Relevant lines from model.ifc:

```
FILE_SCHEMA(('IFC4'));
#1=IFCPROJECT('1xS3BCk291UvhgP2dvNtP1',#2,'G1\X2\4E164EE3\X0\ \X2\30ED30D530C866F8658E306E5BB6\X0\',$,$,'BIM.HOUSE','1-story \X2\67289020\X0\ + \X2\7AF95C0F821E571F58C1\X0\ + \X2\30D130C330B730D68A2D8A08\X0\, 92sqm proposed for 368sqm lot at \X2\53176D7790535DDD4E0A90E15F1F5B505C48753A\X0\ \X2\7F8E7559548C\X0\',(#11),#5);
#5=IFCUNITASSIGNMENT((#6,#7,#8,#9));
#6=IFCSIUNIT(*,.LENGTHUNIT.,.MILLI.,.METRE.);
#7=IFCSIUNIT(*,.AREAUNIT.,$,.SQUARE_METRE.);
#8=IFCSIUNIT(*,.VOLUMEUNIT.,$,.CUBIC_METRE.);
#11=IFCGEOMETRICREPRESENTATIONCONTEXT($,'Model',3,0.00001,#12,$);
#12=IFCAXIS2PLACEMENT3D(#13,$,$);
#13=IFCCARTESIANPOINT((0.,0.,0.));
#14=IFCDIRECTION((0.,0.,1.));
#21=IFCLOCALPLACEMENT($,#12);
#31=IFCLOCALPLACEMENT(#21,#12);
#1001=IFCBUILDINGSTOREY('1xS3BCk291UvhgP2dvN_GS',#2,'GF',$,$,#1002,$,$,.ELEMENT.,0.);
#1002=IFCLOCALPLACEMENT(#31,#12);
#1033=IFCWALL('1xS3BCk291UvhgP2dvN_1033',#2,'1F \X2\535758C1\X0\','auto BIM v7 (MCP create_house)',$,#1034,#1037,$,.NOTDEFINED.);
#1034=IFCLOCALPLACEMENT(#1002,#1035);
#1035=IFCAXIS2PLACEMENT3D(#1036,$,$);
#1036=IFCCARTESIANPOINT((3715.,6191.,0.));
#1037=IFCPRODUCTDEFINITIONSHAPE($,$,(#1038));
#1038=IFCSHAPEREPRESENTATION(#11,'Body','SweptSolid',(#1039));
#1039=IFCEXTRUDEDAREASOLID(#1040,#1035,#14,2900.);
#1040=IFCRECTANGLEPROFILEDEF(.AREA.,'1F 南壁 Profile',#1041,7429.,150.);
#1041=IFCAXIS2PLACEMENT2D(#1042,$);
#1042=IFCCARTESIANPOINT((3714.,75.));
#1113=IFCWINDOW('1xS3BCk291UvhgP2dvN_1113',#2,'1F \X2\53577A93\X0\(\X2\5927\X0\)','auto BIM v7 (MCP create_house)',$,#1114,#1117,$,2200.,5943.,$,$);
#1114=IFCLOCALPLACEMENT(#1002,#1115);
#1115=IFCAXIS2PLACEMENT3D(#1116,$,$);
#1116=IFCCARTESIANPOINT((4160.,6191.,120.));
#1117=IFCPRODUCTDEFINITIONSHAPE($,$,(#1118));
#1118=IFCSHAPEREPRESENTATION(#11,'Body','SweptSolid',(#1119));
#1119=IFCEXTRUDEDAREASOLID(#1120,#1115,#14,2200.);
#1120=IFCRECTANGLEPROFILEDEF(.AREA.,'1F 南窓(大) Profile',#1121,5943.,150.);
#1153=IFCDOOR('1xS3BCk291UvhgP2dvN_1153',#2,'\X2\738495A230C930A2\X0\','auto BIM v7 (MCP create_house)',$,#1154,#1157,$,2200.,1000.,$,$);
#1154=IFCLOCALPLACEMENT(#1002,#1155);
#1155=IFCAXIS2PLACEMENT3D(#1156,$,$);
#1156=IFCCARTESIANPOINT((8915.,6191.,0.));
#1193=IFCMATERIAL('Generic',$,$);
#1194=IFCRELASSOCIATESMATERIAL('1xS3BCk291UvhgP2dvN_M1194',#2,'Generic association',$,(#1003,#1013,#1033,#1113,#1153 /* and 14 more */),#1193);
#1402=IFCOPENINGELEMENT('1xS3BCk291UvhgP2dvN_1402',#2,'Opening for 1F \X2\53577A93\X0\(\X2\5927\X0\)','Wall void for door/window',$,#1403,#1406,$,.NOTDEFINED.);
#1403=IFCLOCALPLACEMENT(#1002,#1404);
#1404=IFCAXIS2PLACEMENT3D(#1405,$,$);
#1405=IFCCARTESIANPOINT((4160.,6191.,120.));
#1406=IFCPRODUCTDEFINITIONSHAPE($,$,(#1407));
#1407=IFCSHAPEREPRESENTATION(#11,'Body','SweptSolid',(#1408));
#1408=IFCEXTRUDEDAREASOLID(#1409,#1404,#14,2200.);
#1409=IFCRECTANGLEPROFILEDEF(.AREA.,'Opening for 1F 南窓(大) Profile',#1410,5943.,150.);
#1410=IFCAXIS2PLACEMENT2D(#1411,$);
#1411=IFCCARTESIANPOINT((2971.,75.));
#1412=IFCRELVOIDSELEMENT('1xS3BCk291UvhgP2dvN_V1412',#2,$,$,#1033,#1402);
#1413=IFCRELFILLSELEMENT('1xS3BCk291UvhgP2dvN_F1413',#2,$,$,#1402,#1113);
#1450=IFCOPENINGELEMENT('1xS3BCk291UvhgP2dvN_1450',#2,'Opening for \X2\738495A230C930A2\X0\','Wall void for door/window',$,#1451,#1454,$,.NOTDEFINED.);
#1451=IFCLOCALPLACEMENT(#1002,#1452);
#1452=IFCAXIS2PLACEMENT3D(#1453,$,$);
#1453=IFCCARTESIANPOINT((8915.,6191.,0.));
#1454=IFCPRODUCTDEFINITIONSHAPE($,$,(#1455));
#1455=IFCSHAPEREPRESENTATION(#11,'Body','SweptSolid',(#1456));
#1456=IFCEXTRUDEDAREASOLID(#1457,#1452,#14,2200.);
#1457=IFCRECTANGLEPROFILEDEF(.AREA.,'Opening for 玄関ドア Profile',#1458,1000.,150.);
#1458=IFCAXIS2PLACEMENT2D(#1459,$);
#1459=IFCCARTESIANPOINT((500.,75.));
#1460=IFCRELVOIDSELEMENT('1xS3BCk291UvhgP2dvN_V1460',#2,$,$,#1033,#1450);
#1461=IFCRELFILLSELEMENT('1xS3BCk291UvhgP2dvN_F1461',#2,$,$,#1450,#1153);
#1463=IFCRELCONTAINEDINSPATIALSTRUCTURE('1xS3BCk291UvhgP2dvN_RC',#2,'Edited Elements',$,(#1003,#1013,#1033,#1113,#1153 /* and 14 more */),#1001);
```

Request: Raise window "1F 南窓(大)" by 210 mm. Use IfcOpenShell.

```python
import numpy as np
import ifcopenshell
import ifcopenshell.api.geometry
import ifcopenshell.util.placement
import ifcopenshell.util.unit

model = ifcopenshell.open("model.ifc")
unit_scale = ifcopenshell.util.unit.calculate_unit_scale(model)

window = model.by_guid("1xS3BCk291UvhgP2dvN_1113")
opening = window.FillsVoids[0].RelatingOpeningElement
dz = 0.21 / unit_scale

shift = np.array([0.0, 0.0, dz])
# The window is not placed relative to its opening, so move both.
for product in (opening, window):
    matrix = ifcopenshell.util.placement.get_local_placement(product.ObjectPlacement)
    matrix[:3, 3] += shift
    ifcopenshell.api.geometry.edit_object_placement(model, product=product, matrix=matrix, is_si=False)

print(f"moved by {dz * unit_scale:+.3f} m")

model.write("model_v2.ifc")
```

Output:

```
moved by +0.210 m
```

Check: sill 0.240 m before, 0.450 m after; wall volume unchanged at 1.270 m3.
